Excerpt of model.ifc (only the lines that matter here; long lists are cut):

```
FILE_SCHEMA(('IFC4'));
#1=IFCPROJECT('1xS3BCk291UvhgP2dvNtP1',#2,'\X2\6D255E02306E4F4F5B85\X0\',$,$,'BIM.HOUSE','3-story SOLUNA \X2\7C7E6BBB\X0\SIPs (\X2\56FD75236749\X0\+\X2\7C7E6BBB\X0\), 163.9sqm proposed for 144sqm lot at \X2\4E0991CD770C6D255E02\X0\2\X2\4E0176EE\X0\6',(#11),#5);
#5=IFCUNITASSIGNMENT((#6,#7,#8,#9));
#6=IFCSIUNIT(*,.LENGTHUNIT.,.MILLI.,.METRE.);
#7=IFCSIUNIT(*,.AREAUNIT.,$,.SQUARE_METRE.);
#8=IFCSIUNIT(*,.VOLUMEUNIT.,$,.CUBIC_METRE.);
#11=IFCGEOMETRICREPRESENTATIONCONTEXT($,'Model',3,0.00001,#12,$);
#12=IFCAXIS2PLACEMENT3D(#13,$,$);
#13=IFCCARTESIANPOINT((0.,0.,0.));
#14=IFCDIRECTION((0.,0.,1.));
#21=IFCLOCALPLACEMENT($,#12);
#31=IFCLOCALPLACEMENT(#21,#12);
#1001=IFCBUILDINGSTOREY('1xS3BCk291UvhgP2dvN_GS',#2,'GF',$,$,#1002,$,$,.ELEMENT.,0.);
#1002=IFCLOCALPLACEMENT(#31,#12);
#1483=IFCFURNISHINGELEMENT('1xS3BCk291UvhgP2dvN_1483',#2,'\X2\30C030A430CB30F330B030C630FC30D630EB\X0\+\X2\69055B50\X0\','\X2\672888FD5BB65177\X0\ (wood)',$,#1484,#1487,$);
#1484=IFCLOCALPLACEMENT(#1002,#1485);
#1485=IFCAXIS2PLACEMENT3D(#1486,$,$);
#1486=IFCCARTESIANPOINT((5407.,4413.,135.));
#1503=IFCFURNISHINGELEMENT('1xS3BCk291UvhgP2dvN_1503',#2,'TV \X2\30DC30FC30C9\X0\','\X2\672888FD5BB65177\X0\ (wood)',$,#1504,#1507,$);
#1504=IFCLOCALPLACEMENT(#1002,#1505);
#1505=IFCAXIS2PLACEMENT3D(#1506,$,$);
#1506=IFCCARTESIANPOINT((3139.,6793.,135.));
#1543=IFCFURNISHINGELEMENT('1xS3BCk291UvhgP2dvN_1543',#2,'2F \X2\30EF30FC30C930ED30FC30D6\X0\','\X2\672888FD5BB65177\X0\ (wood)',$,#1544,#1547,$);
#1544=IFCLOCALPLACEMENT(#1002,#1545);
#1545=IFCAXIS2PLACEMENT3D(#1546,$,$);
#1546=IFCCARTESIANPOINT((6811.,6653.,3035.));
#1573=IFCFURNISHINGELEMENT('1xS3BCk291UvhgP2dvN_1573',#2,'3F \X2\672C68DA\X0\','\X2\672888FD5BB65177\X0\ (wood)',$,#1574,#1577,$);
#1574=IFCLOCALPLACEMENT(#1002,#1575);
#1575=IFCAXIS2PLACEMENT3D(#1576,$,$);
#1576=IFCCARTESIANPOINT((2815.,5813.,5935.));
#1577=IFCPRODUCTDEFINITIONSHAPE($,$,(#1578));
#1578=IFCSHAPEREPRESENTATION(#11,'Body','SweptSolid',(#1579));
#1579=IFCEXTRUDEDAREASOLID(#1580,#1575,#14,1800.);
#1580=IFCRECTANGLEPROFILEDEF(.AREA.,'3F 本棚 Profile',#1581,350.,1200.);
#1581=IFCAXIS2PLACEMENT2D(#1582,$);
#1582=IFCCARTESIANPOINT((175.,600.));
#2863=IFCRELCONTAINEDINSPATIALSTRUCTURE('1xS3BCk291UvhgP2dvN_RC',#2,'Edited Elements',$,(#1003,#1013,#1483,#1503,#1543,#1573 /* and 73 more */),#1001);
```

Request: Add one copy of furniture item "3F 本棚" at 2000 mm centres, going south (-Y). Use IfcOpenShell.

```python
import numpy as np
import ifcopenshell
import ifcopenshell.api.geometry
import ifcopenshell.api.root
import ifcopenshell.util.element
import ifcopenshell.util.placement

model = ifcopenshell.open("model.ifc")


def reuse_history(source, copy):
    """copy_class also copies each property set's owner history, people and application; keep the originals."""
    for rel in copy.IsDefinedBy:
        if rel.is_a("IfcRelDefinesByProperties") and (history := rel.RelatingPropertyDefinition.OwnerHistory):
            rel.RelatingPropertyDefinition.OwnerHistory = source.OwnerHistory
            ifcopenshell.util.element.remove_deep2(model, history)


source = model.by_guid("1xS3BCk291UvhgP2dvN_1573")
base = ifcopenshell.util.placement.get_local_placement(source.ObjectPlacement)
step = np.array([0.0, -1.0, 0.0]) * 2000.0

for i in range(1, 2):
    copy = ifcopenshell.api.root.copy_class(model, product=source)
    copy.Representation = ifcopenshell.util.element.copy_deep(
        model, source.Representation, exclude=["IfcGeometricRepresentationContext", "IfcRepresentationMap"]
    )
    reuse_history(source, copy)
    matrix = base.copy()
    matrix[:3, 3] += i * step
    print("added at", matrix[:3, 3].round(3) + 0.0)
    ifcopenshell.api.geometry.edit_object_placement(model, product=copy, matrix=matrix, is_si=False)

model.write("model-out.ifc")
```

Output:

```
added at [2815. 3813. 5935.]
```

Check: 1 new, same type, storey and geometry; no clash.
